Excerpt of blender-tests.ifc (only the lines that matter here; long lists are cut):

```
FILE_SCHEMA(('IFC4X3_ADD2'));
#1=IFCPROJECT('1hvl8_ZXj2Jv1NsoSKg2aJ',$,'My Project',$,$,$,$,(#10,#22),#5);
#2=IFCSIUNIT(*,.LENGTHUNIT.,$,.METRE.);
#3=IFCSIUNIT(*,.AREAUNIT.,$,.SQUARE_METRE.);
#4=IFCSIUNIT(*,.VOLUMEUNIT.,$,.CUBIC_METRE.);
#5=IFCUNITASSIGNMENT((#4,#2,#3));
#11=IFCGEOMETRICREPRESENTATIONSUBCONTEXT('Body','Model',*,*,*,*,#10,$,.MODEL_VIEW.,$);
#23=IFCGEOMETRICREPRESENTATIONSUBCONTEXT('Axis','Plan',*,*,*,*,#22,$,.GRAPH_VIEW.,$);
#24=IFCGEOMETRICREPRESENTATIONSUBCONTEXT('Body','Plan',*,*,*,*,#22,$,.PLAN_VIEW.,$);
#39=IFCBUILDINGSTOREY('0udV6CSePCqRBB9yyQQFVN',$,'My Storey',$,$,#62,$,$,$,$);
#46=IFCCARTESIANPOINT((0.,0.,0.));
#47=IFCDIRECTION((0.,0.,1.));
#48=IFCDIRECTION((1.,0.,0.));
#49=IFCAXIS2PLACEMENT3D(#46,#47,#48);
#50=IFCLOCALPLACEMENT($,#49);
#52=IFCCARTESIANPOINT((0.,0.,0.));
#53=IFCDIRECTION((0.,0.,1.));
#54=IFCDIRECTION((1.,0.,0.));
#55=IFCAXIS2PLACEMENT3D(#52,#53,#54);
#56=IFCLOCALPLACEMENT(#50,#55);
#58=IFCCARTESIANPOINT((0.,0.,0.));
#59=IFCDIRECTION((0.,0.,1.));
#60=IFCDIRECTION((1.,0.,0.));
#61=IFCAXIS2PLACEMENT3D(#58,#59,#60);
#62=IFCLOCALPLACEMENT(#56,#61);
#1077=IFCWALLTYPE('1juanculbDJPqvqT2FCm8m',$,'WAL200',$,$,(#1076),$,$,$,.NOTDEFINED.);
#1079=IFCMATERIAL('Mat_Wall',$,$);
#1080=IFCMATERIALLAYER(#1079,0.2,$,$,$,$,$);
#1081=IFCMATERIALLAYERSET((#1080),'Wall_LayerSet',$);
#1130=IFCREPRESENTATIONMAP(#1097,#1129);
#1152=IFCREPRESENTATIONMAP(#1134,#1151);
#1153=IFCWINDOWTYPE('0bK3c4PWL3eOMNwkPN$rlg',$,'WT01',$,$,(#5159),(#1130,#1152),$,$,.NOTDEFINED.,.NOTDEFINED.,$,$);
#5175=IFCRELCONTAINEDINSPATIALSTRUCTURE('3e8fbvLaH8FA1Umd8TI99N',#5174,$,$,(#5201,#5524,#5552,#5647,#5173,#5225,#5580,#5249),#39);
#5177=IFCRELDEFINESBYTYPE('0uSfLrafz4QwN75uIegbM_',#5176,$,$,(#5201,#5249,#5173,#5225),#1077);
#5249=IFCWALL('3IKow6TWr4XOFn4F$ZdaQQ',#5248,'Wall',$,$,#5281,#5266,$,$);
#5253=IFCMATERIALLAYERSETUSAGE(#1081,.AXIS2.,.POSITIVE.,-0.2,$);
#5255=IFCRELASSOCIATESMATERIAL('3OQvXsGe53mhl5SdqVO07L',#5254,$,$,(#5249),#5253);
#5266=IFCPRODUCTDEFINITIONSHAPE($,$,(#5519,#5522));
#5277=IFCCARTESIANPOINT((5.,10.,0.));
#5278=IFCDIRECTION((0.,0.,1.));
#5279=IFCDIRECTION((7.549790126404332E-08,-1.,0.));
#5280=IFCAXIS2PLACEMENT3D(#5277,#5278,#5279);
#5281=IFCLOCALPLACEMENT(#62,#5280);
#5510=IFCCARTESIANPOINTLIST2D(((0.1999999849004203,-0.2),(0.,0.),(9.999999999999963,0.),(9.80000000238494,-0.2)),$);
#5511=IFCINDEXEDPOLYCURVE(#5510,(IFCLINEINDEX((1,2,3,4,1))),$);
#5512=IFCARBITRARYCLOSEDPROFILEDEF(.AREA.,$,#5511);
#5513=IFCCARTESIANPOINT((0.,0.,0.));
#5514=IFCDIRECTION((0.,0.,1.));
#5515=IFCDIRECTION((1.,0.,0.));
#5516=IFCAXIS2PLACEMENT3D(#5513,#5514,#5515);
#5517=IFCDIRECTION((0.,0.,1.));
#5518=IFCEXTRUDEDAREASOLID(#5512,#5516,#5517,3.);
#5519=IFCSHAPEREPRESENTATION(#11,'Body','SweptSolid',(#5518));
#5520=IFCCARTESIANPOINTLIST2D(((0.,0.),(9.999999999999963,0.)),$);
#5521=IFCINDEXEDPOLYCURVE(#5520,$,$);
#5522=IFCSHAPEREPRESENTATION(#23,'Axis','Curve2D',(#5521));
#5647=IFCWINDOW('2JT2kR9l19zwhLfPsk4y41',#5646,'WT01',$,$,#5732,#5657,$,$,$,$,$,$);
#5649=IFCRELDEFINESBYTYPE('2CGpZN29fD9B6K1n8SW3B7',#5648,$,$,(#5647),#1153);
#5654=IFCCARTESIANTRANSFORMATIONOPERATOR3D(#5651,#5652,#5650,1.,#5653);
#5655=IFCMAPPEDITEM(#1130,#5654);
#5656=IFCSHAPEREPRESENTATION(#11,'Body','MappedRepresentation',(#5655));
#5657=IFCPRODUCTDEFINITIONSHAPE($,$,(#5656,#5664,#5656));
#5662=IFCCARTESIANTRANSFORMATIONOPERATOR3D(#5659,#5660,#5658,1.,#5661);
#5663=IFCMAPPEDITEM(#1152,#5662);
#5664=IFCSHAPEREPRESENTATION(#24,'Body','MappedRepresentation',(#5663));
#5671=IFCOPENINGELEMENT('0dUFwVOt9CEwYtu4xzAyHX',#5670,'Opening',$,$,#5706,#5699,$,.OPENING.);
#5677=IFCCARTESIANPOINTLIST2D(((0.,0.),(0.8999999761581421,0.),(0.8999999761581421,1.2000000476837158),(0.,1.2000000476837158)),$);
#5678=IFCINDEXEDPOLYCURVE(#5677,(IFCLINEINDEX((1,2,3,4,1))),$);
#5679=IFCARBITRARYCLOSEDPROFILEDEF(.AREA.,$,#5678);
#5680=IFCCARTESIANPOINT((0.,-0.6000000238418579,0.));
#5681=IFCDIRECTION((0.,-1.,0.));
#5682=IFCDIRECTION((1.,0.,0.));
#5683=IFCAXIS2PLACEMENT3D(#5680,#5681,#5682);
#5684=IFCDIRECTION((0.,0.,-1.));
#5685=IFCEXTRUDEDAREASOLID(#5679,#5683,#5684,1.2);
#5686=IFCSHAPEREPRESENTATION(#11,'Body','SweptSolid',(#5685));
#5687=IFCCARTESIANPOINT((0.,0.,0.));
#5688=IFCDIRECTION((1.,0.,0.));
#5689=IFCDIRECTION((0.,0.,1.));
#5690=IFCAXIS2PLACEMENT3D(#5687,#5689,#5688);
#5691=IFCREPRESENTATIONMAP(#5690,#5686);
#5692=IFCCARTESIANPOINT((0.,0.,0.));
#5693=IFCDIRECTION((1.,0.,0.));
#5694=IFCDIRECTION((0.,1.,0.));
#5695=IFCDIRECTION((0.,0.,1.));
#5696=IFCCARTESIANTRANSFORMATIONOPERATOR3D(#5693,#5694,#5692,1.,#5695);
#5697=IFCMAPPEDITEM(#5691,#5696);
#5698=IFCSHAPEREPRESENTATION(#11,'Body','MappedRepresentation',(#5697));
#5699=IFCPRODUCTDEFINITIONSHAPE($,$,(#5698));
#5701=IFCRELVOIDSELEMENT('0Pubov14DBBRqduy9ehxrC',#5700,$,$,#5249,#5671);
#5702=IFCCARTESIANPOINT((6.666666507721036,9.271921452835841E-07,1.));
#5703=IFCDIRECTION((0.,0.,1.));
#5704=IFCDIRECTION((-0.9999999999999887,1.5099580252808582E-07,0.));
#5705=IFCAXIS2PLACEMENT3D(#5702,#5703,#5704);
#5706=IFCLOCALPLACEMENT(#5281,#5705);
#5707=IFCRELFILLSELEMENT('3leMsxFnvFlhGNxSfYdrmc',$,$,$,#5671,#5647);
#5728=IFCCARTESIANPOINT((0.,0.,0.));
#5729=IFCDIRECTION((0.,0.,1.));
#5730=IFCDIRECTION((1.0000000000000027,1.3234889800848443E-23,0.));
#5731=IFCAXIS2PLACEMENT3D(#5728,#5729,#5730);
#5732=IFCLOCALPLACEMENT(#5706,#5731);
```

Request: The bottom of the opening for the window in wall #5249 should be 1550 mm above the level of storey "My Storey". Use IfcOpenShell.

```python
import numpy as np
import ifcopenshell
import ifcopenshell.api.geometry
import ifcopenshell.geom
import ifcopenshell.util.element
import ifcopenshell.util.placement
import ifcopenshell.util.shape
import ifcopenshell.util.unit

model = ifcopenshell.open("blender-tests.ifc")
unit_scale = ifcopenshell.util.unit.calculate_unit_scale(model)

window = model.by_guid("2JT2kR9l19zwhLfPsk4y41")
opening = window.FillsVoids[0].RelatingOpeningElement
storey = ifcopenshell.util.element.get_container(window, ifc_class="IfcBuildingStorey")
level = ifcopenshell.util.placement.get_local_placement(storey.ObjectPlacement)[2, 3]

# The opening's origin need not be at the sill, so measure its lowest point.
shape = ifcopenshell.geom.create_shape(ifcopenshell.geom.settings(), opening)
bottom = ifcopenshell.util.shape.get_shape_bottom_elevation(shape, shape.geometry) / unit_scale
dz = level + 1.55 / unit_scale - bottom

shift = np.array([0.0, 0.0, dz])
# The window is placed relative to its opening, so it follows when the opening moves.
matrix = ifcopenshell.util.placement.get_local_placement(opening.ObjectPlacement)
matrix[:3, 3] += shift
ifcopenshell.api.geometry.edit_object_placement(
    model, product=opening, matrix=matrix, is_si=False, should_transform_children=True
)

print(f"moved by {dz * unit_scale:+.3f} m")

model.write("blender-tests-out.ifc")
```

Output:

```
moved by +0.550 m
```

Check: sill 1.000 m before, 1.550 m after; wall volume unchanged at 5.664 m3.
